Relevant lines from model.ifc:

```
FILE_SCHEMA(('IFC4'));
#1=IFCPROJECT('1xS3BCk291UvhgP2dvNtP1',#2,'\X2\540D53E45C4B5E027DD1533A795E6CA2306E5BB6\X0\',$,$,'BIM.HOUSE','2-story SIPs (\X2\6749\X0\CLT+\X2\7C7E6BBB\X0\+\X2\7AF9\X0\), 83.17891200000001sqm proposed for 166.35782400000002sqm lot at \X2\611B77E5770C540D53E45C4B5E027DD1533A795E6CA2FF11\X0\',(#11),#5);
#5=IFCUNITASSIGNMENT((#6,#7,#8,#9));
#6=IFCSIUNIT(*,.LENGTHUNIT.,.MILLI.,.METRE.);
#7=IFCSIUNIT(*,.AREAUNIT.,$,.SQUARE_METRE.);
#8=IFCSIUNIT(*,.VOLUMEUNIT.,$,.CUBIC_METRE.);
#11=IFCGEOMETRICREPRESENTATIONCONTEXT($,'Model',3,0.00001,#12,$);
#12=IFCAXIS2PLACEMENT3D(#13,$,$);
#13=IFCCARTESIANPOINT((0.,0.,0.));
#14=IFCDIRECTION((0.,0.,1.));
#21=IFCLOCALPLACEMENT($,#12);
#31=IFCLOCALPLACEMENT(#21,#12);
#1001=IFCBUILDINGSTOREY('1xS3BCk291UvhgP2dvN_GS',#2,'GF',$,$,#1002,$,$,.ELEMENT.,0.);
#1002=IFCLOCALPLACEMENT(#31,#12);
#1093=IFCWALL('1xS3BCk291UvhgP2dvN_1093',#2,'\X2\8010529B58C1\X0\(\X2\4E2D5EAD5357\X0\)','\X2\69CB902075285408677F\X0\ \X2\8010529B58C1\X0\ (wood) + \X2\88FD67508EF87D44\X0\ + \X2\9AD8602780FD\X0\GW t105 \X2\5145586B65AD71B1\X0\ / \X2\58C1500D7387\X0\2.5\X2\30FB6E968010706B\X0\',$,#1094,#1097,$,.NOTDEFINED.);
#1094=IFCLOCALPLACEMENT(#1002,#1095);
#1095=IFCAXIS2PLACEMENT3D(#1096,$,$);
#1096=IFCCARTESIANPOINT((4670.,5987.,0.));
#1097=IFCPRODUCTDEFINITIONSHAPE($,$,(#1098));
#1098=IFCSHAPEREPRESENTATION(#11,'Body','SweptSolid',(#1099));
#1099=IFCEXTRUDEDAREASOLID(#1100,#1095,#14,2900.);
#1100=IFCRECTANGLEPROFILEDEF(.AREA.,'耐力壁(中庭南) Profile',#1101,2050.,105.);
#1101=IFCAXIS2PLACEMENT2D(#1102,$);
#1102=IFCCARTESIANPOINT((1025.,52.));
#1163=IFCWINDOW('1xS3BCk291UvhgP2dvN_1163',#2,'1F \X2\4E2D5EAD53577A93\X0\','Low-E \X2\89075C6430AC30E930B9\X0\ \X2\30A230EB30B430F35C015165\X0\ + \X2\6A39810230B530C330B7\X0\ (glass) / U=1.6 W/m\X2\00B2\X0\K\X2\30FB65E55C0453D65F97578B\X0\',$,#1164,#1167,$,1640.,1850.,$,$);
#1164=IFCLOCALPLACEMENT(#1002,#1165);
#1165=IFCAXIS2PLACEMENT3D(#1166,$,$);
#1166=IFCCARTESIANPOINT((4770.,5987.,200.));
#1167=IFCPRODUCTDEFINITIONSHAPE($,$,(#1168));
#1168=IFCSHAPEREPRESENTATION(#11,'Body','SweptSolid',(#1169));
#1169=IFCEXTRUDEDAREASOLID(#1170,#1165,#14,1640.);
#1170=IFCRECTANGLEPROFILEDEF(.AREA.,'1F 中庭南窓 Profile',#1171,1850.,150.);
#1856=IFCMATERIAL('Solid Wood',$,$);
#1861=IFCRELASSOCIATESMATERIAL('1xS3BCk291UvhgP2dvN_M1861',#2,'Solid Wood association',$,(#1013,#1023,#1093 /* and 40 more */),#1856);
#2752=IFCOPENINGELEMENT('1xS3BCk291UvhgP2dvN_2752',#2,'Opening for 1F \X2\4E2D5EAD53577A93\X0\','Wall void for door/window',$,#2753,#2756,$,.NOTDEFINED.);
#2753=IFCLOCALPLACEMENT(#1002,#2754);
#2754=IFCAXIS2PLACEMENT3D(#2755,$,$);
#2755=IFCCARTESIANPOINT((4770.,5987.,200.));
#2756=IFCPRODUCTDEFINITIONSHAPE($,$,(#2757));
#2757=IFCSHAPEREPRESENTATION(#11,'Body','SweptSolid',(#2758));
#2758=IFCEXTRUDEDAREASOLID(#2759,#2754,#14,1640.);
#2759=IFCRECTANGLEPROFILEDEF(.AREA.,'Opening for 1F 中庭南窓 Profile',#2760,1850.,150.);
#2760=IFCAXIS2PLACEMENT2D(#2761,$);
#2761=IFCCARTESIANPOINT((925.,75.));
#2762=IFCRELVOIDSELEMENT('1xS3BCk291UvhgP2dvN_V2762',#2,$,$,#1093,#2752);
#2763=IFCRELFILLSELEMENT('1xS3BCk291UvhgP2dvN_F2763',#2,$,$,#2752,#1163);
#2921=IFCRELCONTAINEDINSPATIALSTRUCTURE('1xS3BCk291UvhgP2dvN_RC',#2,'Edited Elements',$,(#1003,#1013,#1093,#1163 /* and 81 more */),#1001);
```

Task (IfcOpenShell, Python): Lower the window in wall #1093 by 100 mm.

```python
import numpy as np
import ifcopenshell
import ifcopenshell.api.geometry
import ifcopenshell.util.placement
import ifcopenshell.util.unit

model = ifcopenshell.open("model.ifc")
unit_scale = ifcopenshell.util.unit.calculate_unit_scale(model)

window = model.by_guid("1xS3BCk291UvhgP2dvN_1163")
opening = window.FillsVoids[0].RelatingOpeningElement
dz = -100.0

shift = np.array([0.0, 0.0, dz])
# The window is not placed relative to its opening, so move both.
for product in (opening, window):
    matrix = ifcopenshell.util.placement.get_local_placement(product.ObjectPlacement)
    matrix[:3, 3] += shift
    ifcopenshell.api.geometry.edit_object_placement(model, product=product, matrix=matrix, is_si=False)

print(f"moved by {dz * unit_scale:+.3f} m")

model.write("model-out.ifc")
```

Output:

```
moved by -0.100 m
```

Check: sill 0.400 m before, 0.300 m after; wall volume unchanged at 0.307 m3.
